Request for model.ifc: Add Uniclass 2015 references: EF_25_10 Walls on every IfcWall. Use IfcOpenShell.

First a look at what the model holds.

```python
import ifcopenshell

model = ifcopenshell.open("model.ifc")
print(model.schema)
print("classifications:", [c.Name for c in model.by_type("IfcClassification")])
for ifc_class in ("IfcDoor", "IfcRoof", "IfcStair", "IfcWall", "IfcWindow"):
    print(ifc_class, len(model.by_type(ifc_class)))
```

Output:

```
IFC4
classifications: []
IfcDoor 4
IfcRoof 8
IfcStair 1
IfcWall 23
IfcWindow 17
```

```python
import ifcopenshell
import ifcopenshell.api.classification

model = ifcopenshell.open("model.ifc")

system = ifcopenshell.api.classification.add_classification(model, classification="Uniclass 2015")

codes = {
    "IfcWall": ("EF_25_10", "Walls"),
}
for ifc_class, (code, name) in codes.items():
    products = model.by_type(ifc_class)
    ifcopenshell.api.classification.add_reference(
        model, products=products, classification=system, identification=code, name=name
    )
    print(code, len(products))

model.write("model_updated.ifc")
```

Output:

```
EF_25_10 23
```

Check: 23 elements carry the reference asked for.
